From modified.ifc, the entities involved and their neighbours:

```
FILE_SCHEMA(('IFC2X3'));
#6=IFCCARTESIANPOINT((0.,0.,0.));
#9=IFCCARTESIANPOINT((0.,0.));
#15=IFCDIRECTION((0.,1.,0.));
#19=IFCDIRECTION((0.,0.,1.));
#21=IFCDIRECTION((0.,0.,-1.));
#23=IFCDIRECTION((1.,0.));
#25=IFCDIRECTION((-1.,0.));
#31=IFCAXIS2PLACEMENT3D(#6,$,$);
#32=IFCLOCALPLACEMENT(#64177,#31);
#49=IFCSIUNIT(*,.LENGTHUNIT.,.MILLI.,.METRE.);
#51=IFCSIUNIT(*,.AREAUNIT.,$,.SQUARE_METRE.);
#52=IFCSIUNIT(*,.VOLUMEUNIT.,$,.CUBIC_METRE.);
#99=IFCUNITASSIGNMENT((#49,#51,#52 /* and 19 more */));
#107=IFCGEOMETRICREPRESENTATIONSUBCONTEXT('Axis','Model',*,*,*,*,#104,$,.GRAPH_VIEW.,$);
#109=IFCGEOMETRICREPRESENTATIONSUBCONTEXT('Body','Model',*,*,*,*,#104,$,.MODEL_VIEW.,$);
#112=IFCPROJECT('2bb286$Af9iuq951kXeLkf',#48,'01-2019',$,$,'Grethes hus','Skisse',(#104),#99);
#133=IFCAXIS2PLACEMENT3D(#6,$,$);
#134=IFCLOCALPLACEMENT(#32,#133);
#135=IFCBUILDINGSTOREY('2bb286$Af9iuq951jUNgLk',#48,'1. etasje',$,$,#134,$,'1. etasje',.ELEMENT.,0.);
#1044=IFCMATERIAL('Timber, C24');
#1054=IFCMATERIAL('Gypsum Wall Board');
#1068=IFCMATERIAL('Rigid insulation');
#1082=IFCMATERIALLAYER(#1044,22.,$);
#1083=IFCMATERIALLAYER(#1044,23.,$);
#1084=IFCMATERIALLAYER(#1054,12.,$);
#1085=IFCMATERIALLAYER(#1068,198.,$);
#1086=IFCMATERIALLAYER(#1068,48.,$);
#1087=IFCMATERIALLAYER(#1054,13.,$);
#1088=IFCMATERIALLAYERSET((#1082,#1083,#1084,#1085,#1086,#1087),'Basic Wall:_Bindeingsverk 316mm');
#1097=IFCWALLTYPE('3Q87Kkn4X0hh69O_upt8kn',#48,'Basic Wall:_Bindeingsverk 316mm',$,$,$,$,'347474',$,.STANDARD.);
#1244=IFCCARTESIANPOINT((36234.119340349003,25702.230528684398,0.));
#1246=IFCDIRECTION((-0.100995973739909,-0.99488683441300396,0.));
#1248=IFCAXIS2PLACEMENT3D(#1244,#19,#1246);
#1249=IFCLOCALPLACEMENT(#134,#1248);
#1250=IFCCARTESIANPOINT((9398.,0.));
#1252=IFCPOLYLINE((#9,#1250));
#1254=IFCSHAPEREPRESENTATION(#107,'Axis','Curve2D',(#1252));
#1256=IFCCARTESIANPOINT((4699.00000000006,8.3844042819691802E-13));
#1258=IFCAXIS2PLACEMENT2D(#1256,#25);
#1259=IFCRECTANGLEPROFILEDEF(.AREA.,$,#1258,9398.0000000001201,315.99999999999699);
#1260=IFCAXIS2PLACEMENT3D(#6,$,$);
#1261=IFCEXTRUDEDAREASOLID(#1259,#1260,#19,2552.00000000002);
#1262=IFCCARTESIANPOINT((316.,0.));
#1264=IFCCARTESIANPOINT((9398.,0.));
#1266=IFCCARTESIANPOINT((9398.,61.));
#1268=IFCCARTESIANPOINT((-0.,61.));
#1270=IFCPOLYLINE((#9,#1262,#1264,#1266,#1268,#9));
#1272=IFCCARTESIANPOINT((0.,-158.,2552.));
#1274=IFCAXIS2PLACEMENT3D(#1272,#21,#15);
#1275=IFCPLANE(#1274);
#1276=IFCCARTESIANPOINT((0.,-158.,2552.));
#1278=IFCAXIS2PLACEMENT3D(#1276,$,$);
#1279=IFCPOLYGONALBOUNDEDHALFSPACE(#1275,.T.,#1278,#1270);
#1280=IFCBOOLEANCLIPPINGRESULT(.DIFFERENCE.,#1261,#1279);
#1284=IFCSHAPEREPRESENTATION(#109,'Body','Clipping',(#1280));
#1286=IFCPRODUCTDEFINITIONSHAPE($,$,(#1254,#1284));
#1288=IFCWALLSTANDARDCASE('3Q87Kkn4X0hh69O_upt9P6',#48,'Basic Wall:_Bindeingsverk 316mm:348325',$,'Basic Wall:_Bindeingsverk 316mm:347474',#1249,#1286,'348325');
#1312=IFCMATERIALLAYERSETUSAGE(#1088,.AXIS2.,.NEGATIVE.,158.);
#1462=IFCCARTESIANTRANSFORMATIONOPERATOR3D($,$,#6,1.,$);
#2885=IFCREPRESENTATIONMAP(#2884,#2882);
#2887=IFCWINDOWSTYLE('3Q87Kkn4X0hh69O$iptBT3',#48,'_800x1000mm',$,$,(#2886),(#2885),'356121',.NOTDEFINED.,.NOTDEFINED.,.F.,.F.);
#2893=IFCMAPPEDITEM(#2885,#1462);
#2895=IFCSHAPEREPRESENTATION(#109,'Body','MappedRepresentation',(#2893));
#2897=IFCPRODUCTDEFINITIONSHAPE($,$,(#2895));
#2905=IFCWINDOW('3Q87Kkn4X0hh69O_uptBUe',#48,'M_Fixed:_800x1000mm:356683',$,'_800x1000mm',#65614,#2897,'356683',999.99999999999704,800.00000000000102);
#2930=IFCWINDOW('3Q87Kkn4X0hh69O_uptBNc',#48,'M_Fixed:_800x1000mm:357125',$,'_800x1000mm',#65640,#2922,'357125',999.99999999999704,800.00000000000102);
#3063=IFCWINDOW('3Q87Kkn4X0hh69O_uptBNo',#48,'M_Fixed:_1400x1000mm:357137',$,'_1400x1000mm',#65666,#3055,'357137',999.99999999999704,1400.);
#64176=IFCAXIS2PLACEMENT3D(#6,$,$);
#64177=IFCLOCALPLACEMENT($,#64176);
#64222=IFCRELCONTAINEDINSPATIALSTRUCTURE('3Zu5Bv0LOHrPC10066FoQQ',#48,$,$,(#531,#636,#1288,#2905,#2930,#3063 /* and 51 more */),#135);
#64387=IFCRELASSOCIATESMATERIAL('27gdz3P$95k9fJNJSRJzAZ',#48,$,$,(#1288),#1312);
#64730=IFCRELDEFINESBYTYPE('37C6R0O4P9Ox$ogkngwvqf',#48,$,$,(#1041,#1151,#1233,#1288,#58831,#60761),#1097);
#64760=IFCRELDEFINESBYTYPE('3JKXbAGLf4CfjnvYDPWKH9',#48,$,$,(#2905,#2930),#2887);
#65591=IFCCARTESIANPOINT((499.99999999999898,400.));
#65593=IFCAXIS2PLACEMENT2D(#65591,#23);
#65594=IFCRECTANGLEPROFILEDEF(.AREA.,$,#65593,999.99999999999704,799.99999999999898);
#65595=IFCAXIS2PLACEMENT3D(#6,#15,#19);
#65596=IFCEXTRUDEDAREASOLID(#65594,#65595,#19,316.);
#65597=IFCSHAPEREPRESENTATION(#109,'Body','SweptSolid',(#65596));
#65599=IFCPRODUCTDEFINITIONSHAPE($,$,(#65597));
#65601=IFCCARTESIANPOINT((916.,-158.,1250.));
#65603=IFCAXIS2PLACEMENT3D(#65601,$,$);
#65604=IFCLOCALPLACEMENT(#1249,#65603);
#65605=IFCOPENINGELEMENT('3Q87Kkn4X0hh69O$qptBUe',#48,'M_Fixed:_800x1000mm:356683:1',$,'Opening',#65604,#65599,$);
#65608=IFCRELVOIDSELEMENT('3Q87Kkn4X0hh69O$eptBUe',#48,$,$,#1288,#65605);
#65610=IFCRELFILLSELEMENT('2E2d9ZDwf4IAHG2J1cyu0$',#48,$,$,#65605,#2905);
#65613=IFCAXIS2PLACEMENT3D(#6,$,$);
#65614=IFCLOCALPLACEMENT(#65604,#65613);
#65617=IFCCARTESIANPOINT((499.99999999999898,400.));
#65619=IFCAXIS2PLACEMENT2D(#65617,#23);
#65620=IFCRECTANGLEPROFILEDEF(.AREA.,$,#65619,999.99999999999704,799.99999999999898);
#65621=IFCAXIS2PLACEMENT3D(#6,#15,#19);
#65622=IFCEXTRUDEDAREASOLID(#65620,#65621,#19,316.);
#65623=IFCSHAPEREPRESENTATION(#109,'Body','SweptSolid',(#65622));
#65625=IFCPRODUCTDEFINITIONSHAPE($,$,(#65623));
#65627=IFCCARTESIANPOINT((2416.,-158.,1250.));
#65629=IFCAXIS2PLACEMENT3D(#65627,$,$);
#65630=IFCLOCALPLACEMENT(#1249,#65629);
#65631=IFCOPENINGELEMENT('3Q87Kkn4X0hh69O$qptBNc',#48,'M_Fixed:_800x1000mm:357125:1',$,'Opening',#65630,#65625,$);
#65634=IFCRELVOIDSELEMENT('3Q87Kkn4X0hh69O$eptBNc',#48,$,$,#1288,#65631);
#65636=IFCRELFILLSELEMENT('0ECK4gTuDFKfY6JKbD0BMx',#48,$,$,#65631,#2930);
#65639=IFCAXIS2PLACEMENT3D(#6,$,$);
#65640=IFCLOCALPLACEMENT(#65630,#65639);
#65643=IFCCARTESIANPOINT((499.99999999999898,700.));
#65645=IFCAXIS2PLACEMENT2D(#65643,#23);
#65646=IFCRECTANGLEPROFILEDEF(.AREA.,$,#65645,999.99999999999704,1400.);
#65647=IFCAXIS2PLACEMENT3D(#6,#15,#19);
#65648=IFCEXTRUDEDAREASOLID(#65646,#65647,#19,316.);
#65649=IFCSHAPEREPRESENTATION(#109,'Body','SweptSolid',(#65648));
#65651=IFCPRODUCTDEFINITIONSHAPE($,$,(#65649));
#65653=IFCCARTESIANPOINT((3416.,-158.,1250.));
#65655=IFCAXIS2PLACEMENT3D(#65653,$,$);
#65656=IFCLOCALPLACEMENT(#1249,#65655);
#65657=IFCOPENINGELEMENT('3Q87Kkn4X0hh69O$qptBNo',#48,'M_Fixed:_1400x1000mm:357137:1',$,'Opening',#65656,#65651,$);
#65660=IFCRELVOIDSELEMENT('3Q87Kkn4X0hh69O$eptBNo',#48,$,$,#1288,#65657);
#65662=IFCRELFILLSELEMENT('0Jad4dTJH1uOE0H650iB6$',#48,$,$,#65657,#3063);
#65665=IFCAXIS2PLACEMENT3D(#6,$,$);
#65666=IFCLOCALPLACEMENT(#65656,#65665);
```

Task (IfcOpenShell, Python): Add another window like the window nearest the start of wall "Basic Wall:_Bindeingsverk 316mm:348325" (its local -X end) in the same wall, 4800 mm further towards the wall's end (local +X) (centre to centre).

```python
import ifcopenshell
import ifcopenshell.api.feature
import ifcopenshell.api.geometry
import ifcopenshell.api.root
import ifcopenshell.geom
import ifcopenshell.util.element
import ifcopenshell.util.placement
import ifcopenshell.util.shape

model = ifcopenshell.open("modified.ifc")
settings = ifcopenshell.geom.settings()


def volume(element):
    """Net volume in cubic metres, openings subtracted."""
    shape = ifcopenshell.geom.create_shape(settings, element)
    return ifcopenshell.util.shape.get_volume(shape.geometry)


def reuse_history(source, copy):
    """copy_class also copies each property set's owner history, people and application; keep the originals."""
    for rel in copy.IsDefinedBy:
        if rel.is_a("IfcRelDefinesByProperties") and (history := rel.RelatingPropertyDefinition.OwnerHistory):
            rel.RelatingPropertyDefinition.OwnerHistory = source.OwnerHistory
            ifcopenshell.util.element.remove_deep2(model, history)


window = model.by_guid("3Q87Kkn4X0hh69O_uptBUe")
opening = window.FillsVoids[0].RelatingOpeningElement
wall = opening.VoidsElements[0].RelatingBuildingElement
before = volume(wall)
shift = ifcopenshell.util.placement.get_local_placement(wall.ObjectPlacement)[:3, 0] * 4800.0

# copy_class copies the void relationship, type, container and properties, but no geometry.
new_opening = ifcopenshell.api.root.copy_class(model, product=opening)
new_opening.Representation = ifcopenshell.util.element.copy_deep(
    model, opening.Representation, exclude=["IfcGeometricRepresentationContext", "IfcRepresentationMap"]
)
new_opening.Name = "M_Fixed:_800x1000mm"
new_window = ifcopenshell.api.root.copy_class(model, product=window)
new_window.Representation = ifcopenshell.util.element.copy_deep(
    model, window.Representation, exclude=["IfcGeometricRepresentationContext", "IfcRepresentationMap"]
)
new_window.Name = "M_Fixed:_800x1000mm"
new_window.Tag = None
reuse_history(window, new_window)
fills = ifcopenshell.api.feature.add_filling(model, opening=new_opening, element=new_window)
fills.OwnerHistory = new_window.OwnerHistory  # required in IFC2X3

for old, new in ((opening, new_opening), (window, new_window)):
    matrix = ifcopenshell.util.placement.get_local_placement(old.ObjectPlacement)
    matrix[:3, 3] += shift
    ifcopenshell.api.geometry.edit_object_placement(model, product=new, matrix=matrix, is_si=False)

after = volume(wall)

print(f"wall volume {before:.3f} -> {after:.3f} m3")

model.write("modified_v2.ifc")
```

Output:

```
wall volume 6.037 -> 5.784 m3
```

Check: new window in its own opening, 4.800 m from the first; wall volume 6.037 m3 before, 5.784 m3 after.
